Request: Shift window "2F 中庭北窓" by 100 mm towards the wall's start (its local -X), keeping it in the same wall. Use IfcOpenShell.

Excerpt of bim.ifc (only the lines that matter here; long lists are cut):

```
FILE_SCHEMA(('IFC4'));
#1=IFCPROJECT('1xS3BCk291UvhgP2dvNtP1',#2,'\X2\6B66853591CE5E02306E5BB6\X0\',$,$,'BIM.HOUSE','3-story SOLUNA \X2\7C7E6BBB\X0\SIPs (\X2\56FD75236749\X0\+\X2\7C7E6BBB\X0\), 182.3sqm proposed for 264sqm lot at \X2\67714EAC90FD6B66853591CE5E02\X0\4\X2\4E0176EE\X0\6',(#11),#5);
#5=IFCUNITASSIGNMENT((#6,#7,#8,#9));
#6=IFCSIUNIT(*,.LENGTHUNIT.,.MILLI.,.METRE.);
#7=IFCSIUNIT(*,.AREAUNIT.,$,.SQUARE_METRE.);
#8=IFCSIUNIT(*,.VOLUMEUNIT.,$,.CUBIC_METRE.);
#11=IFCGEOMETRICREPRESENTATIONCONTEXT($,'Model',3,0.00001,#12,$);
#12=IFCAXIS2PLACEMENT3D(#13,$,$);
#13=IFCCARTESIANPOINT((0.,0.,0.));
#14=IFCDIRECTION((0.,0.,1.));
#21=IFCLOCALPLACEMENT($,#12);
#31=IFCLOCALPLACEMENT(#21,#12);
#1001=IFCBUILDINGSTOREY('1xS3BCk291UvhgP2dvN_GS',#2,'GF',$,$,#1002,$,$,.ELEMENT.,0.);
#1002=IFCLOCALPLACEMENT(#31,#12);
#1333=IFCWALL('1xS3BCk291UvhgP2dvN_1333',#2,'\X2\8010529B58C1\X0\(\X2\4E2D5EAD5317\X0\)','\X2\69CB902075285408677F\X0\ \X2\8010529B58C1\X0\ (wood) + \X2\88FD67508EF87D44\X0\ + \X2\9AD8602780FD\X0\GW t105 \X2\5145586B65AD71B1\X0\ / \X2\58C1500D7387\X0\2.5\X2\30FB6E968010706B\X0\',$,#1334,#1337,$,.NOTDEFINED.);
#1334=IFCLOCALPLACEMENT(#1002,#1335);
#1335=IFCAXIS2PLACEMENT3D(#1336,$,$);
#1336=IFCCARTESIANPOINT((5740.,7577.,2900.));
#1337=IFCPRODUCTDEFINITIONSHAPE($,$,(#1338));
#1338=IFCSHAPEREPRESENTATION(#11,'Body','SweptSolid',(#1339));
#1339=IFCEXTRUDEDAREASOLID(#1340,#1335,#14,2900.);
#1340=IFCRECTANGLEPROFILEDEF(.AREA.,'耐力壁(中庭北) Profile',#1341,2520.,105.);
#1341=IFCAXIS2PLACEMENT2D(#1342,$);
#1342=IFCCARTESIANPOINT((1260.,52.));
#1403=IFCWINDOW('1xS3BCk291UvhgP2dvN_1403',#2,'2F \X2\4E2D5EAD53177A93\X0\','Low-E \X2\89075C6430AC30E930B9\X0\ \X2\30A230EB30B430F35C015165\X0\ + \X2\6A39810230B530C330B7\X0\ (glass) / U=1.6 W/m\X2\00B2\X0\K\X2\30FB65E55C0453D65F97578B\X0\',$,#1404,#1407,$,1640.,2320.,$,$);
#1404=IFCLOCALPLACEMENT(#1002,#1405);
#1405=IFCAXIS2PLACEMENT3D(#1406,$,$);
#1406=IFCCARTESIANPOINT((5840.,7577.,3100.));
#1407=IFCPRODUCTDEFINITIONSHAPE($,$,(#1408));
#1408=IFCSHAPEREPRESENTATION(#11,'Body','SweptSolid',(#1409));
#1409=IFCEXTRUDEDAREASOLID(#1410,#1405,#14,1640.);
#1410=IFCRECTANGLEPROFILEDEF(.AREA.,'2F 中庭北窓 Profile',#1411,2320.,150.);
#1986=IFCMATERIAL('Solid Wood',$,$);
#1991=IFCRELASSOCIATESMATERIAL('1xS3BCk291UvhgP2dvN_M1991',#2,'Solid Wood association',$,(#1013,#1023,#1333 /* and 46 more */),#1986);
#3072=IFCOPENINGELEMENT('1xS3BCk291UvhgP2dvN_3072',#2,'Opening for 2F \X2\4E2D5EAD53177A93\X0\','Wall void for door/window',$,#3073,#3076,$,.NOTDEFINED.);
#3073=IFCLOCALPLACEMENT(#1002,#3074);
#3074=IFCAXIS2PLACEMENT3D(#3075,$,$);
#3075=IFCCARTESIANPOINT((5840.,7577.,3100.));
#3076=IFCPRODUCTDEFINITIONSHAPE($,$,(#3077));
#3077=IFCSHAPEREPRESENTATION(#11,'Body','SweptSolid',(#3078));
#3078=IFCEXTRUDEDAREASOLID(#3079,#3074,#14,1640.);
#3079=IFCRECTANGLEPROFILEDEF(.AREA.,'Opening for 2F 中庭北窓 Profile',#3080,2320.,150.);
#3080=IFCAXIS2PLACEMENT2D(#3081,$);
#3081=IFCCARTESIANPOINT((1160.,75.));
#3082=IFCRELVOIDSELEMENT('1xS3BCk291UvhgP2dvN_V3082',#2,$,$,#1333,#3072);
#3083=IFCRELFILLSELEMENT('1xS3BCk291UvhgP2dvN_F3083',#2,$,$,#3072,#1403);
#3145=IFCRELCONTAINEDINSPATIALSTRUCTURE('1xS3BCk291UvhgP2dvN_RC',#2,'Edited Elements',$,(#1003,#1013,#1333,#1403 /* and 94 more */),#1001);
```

```python
import ifcopenshell
import ifcopenshell.api.geometry
import ifcopenshell.util.placement

model = ifcopenshell.open("bim.ifc")

window = model.by_guid("1xS3BCk291UvhgP2dvN_1403")
opening = window.FillsVoids[0].RelatingOpeningElement
wall = opening.VoidsElements[0].RelatingBuildingElement

wall_matrix = ifcopenshell.util.placement.get_local_placement(wall.ObjectPlacement)
shift = wall_matrix[:3, 0] * -100.0
before = ifcopenshell.util.placement.get_local_placement(window.ObjectPlacement)[:3, 3].copy()

# The window is not placed relative to its opening, so move both.
for product in (opening, window):
    matrix = ifcopenshell.util.placement.get_local_placement(product.ObjectPlacement)
    matrix[:3, 3] += shift
    ifcopenshell.api.geometry.edit_object_placement(model, product=product, matrix=matrix, is_si=False)

after = ifcopenshell.util.placement.get_local_placement(window.ObjectPlacement)[:3, 3]
print("window moved by", (after - before).round(3) + 0.0)

model.write("bim_v2.ifc")
```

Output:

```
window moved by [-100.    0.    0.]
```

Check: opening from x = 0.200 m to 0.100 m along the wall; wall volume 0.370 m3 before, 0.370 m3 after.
